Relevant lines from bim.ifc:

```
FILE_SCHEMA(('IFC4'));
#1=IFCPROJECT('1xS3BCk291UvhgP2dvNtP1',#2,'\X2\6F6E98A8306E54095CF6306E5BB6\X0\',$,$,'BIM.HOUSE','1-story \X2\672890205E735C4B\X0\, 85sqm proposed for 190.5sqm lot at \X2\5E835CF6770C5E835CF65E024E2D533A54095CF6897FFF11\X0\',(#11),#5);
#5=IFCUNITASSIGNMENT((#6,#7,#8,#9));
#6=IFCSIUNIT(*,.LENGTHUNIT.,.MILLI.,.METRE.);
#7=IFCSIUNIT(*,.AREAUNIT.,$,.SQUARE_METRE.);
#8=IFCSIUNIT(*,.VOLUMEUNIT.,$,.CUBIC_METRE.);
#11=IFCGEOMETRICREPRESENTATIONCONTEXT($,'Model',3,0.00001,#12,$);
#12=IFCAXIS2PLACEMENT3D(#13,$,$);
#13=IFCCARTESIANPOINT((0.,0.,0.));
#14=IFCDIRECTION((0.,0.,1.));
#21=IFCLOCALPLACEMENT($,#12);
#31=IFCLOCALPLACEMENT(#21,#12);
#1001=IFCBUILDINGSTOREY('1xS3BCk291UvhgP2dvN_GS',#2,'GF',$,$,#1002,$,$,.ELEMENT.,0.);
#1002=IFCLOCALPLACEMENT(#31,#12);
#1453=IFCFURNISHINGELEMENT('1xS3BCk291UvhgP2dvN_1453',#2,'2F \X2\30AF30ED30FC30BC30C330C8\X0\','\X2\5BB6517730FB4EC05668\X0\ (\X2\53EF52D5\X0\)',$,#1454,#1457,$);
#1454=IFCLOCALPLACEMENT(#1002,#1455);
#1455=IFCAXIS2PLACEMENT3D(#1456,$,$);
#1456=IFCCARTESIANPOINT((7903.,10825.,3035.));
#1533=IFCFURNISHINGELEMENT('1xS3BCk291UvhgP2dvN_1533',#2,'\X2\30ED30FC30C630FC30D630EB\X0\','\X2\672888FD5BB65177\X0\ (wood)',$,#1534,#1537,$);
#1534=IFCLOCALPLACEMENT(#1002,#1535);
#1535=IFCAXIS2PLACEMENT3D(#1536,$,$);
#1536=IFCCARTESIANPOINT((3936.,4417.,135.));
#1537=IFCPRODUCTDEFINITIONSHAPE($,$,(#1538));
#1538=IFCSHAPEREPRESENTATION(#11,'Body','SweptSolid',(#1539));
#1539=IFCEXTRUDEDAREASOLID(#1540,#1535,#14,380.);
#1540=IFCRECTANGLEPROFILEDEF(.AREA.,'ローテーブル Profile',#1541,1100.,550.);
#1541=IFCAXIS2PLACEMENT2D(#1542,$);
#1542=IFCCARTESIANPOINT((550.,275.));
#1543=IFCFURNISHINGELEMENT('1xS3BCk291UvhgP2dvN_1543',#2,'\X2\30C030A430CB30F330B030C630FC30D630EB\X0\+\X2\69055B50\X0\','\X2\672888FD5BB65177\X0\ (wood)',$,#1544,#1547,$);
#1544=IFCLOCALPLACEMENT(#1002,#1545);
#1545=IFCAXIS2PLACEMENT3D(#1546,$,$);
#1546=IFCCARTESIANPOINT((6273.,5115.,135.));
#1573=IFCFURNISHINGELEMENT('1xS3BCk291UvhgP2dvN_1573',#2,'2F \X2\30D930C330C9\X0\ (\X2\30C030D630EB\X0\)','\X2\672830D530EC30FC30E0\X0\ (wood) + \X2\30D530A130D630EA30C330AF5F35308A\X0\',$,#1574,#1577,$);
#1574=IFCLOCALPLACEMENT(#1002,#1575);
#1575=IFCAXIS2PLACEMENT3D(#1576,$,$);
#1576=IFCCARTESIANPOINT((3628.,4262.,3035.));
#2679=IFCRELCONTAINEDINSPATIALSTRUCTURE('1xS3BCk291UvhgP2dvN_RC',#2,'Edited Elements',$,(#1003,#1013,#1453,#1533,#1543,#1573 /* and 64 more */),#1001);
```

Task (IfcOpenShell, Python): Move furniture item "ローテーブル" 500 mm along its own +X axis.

```python
import ifcopenshell
import ifcopenshell.api.geometry
import ifcopenshell.util.placement
import ifcopenshell.util.unit

model = ifcopenshell.open("bim.ifc")
unit_scale = ifcopenshell.util.unit.calculate_unit_scale(model)

item = model.by_guid("1xS3BCk291UvhgP2dvN_1533")
matrix = ifcopenshell.util.placement.get_local_placement(item.ObjectPlacement)
matrix[:3, 3] += matrix[:3, 0] * 0.5 / unit_scale
ifcopenshell.api.geometry.edit_object_placement(model, product=item, matrix=matrix, is_si=False)

print(ifcopenshell.util.placement.get_local_placement(item.ObjectPlacement).round(3) + 0.0)

model.write("bim_updated.ifc")
```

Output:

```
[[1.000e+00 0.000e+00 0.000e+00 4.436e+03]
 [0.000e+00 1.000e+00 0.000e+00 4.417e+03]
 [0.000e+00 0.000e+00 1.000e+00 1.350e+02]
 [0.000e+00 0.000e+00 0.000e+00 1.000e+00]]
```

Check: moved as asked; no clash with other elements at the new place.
